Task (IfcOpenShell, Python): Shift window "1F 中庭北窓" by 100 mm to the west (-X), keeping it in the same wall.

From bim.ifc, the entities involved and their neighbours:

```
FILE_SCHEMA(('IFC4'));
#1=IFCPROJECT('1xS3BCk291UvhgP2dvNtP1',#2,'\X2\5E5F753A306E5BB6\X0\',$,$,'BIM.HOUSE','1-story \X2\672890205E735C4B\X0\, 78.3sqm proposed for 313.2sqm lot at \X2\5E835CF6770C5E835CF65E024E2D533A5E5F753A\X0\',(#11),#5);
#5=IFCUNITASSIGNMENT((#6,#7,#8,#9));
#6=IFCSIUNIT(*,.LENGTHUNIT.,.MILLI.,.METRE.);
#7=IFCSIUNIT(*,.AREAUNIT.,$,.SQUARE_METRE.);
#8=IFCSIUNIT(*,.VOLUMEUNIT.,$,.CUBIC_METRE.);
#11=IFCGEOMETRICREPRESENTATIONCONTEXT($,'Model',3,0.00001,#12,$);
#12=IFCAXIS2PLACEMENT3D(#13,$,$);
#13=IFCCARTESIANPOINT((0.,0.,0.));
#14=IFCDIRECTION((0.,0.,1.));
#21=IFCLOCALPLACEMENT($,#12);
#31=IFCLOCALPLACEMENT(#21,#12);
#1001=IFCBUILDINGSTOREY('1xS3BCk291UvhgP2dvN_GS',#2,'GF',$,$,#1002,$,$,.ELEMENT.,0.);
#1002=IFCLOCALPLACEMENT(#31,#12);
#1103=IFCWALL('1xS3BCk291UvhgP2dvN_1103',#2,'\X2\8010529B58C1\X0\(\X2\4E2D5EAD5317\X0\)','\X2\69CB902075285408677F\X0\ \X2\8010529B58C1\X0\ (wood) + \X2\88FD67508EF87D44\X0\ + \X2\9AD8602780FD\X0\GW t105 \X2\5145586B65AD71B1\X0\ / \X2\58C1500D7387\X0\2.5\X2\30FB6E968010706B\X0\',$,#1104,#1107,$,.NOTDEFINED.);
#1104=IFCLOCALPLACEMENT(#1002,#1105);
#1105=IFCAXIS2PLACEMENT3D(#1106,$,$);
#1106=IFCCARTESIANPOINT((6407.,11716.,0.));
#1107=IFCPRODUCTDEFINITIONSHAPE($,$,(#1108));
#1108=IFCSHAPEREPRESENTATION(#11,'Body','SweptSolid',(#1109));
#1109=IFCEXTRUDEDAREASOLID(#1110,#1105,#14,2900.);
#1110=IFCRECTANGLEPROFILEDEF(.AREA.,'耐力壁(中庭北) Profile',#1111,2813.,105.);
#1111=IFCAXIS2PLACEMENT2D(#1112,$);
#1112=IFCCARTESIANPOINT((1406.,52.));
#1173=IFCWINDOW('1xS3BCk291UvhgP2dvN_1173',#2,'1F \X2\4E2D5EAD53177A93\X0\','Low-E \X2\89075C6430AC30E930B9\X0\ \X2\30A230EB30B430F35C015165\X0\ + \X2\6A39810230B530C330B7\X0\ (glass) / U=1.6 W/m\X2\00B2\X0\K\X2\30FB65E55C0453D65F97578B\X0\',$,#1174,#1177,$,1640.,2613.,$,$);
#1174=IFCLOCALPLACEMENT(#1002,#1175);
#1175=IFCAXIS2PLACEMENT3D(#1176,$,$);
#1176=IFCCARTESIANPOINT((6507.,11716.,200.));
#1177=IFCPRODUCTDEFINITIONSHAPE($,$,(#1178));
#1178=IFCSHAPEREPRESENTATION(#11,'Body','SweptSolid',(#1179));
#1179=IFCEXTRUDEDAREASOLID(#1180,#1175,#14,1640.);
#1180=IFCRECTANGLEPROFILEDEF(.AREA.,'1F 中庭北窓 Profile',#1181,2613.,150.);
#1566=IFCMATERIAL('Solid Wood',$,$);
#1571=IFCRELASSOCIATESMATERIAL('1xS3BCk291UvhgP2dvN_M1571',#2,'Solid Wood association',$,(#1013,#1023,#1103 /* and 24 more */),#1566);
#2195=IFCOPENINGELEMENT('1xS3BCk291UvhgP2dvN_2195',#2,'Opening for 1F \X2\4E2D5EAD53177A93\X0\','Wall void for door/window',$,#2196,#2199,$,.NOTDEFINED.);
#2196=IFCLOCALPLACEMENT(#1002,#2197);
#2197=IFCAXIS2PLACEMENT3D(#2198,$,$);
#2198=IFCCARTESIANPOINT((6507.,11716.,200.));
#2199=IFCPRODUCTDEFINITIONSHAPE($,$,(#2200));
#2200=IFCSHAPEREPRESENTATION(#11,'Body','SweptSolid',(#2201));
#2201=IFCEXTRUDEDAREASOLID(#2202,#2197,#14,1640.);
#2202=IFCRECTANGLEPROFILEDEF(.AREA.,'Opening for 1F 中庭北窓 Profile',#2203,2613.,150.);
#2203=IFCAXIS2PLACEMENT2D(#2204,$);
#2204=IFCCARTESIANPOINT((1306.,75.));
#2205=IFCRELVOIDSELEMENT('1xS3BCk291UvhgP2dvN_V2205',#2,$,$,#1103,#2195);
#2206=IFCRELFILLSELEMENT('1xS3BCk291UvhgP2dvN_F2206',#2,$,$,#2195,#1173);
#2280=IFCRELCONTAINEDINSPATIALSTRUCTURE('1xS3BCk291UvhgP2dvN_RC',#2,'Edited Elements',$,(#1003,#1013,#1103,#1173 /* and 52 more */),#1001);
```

```python
import ifcopenshell
import ifcopenshell.api.geometry
import ifcopenshell.util.placement
import ifcopenshell.util.unit

model = ifcopenshell.open("bim.ifc")
unit_scale = ifcopenshell.util.unit.calculate_unit_scale(model)

window = model.by_guid("1xS3BCk291UvhgP2dvN_1173")
opening = window.FillsVoids[0].RelatingOpeningElement
wall = opening.VoidsElements[0].RelatingBuildingElement

wall_matrix = ifcopenshell.util.placement.get_local_placement(wall.ObjectPlacement)
shift = wall_matrix[:3, 0] * -0.1 / unit_scale
before = ifcopenshell.util.placement.get_local_placement(window.ObjectPlacement)[:3, 3].copy()

# The window is not placed relative to its opening, so move both.
for product in (opening, window):
    matrix = ifcopenshell.util.placement.get_local_placement(product.ObjectPlacement)
    matrix[:3, 3] += shift
    ifcopenshell.api.geometry.edit_object_placement(model, product=product, matrix=matrix, is_si=False)

after = ifcopenshell.util.placement.get_local_placement(window.ObjectPlacement)[:3, 3]
print("window moved by", (after - before).round(3) + 0.0)

model.write("bim_rev.ifc")
```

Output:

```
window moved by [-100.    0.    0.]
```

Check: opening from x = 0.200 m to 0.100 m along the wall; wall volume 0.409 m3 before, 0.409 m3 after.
